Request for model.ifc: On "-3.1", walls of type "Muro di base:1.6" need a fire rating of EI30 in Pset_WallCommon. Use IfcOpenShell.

First a look at what the model holds.

```python
import ifcopenshell
import ifcopenshell.util.element

model = ifcopenshell.open("model.ifc")
print(model.schema)
storey = next(s for s in model.by_type("IfcBuildingStorey") if s.Name == "-3.1")
walls = [e for e in ifcopenshell.util.element.get_decomposition(storey) if e.is_a("IfcWall")]
seen = {}
for e in walls:
    element_type = ifcopenshell.util.element.get_type(e)
    key = (element_type.Name if element_type != e and element_type else None, ifcopenshell.util.element.get_pset(e, "Pset_WallCommon", "FireRating"))
    seen[key] = seen.get(key, 0) + 1
for (name, value), count in sorted(seen.items(), key=str):
    print(count, "x", name, "|", value)
```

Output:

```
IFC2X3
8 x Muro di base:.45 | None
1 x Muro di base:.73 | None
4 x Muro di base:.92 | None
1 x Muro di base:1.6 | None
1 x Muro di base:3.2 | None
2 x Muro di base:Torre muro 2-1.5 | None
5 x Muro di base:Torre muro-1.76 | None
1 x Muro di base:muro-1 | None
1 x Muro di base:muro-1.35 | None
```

```python
import ifcopenshell
import ifcopenshell.api.pset
import ifcopenshell.util.element

model = ifcopenshell.open("model.ifc")

storey = next(s for s in model.by_type("IfcBuildingStorey") if s.Name == "-3.1")
walls = [e for e in ifcopenshell.util.element.get_decomposition(storey) if e.is_a("IfcWall")]

count = 0
for e in walls:
    element_type = ifcopenshell.util.element.get_type(e)
    if element_type in (None, e) or element_type.Name != "Muro di base:1.6":
        continue
    # add_pset returns the element's existing set when there is one.
    pset = ifcopenshell.api.pset.add_pset(model, product=e, name="Pset_WallCommon")
    ifcopenshell.api.pset.edit_pset(model, pset=pset, properties={"FireRating": "EI30"})
    count += 1

print(count, "walls updated")

model.write("model-out.ifc")
```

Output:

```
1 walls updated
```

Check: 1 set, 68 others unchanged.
